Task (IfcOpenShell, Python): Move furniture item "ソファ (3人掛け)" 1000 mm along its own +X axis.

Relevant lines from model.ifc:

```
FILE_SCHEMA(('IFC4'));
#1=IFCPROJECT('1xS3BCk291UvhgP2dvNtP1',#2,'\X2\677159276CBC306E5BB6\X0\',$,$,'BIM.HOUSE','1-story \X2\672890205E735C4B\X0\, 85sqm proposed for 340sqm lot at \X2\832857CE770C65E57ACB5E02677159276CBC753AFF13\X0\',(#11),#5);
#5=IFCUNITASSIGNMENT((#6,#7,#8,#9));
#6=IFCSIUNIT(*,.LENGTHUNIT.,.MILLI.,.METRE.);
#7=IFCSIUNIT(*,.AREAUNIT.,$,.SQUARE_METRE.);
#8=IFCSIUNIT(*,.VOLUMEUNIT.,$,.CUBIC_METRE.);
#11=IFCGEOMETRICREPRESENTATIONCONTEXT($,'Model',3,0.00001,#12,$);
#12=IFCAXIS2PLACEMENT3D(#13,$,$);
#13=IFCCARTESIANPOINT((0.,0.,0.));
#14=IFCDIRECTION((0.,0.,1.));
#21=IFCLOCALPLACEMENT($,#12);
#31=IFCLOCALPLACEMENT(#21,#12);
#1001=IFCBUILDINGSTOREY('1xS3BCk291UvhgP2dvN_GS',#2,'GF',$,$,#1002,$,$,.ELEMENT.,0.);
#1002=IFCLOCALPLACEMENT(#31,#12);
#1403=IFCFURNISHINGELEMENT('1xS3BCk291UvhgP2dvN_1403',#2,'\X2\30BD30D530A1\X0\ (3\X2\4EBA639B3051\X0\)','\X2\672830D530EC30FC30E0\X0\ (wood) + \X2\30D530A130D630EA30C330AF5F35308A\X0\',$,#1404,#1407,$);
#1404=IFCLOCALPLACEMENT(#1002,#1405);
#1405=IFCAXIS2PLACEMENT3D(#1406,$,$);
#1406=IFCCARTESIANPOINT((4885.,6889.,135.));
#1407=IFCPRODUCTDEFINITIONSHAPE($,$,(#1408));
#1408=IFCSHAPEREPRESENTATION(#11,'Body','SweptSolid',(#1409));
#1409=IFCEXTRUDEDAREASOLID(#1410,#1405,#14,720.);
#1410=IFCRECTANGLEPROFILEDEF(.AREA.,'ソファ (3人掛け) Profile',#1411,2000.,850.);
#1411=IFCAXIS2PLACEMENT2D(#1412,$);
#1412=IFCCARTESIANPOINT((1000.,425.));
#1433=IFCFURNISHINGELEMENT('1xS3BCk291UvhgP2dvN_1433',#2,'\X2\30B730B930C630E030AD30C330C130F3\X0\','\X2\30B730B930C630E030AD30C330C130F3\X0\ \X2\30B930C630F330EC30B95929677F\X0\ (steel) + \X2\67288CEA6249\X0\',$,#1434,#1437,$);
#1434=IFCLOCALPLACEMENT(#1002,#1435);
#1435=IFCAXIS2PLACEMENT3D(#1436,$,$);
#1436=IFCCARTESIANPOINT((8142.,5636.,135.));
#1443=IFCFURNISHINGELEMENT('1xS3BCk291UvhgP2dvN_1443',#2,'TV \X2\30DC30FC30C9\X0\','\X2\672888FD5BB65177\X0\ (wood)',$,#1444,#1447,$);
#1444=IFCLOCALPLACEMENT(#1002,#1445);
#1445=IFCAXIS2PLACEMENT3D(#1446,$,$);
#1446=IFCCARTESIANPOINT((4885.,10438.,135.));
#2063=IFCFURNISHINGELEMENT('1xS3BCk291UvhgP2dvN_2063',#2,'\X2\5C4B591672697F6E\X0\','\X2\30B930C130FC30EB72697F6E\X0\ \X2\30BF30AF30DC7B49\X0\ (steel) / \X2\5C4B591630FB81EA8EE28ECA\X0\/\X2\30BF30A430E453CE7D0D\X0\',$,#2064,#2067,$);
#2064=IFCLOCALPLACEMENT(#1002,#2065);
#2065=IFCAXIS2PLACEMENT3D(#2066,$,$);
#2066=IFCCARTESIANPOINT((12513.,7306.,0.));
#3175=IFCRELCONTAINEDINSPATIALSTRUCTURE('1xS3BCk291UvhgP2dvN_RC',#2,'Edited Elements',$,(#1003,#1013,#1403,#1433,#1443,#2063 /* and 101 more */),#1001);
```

```python
import ifcopenshell
import ifcopenshell.api.geometry
import ifcopenshell.util.placement

model = ifcopenshell.open("model.ifc")

item = model.by_guid("1xS3BCk291UvhgP2dvN_1403")
matrix = ifcopenshell.util.placement.get_local_placement(item.ObjectPlacement)
matrix[:3, 3] += matrix[:3, 0] * 1000.0
ifcopenshell.api.geometry.edit_object_placement(model, product=item, matrix=matrix, is_si=False)

print(ifcopenshell.util.placement.get_local_placement(item.ObjectPlacement).round(3) + 0.0)

model.write("model-out.ifc")
```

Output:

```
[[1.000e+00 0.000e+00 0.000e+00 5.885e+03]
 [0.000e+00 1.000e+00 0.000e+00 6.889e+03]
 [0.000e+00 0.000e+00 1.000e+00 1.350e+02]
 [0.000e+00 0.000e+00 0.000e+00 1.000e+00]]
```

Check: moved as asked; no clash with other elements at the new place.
